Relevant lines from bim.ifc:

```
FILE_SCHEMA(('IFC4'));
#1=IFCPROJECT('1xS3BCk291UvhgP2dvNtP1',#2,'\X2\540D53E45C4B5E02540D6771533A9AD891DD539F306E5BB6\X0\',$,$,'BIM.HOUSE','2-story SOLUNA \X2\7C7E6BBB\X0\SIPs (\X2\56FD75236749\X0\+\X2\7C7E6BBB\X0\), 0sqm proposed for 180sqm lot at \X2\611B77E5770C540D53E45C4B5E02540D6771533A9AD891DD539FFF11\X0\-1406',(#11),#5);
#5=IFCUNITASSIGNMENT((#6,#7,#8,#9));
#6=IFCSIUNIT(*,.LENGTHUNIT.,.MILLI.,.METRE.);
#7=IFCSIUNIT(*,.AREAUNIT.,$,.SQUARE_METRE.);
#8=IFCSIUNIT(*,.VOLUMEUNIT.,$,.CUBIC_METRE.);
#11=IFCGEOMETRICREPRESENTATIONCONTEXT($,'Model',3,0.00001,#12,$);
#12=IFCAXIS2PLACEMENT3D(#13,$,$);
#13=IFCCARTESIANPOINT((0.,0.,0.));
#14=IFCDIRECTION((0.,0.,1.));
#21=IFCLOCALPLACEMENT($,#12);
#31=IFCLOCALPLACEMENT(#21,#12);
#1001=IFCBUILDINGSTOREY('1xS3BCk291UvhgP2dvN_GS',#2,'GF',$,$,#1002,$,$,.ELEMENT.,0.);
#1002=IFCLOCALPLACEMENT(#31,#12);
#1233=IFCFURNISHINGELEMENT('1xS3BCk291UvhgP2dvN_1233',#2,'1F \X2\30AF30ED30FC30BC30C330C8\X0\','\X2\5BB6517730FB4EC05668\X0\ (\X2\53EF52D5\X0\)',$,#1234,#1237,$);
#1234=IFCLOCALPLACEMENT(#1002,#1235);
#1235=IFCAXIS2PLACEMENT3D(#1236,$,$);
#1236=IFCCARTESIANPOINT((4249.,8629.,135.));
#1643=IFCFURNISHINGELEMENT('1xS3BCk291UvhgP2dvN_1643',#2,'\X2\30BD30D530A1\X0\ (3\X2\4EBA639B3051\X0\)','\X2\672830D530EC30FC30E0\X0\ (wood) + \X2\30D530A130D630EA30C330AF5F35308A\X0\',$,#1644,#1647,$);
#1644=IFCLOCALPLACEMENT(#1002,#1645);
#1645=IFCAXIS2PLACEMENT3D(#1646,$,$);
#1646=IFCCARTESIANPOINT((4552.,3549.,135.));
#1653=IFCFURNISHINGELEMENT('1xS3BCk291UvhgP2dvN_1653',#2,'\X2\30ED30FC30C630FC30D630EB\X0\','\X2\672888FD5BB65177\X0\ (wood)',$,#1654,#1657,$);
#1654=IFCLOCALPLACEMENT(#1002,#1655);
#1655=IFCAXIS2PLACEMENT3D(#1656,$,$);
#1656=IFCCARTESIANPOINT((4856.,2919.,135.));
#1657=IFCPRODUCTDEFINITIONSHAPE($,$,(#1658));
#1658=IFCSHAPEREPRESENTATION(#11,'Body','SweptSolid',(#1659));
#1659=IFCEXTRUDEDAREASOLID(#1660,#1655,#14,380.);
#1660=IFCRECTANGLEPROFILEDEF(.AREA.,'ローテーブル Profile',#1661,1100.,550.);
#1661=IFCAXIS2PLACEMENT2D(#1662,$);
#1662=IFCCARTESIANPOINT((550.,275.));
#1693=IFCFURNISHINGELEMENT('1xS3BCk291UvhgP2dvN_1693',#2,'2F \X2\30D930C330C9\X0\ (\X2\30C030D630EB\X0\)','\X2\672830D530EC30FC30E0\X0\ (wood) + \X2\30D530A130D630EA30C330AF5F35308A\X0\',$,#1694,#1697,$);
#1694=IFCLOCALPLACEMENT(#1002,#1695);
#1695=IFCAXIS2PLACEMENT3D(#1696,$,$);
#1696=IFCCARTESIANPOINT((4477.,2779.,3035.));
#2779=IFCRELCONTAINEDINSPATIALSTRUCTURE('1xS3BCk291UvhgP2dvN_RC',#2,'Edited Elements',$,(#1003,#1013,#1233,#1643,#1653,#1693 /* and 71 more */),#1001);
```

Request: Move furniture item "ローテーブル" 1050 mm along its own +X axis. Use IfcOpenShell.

```python
import ifcopenshell
import ifcopenshell.api.geometry
import ifcopenshell.util.placement
import ifcopenshell.util.unit

model = ifcopenshell.open("bim.ifc")
unit_scale = ifcopenshell.util.unit.calculate_unit_scale(model)

item = model.by_guid("1xS3BCk291UvhgP2dvN_1653")
matrix = ifcopenshell.util.placement.get_local_placement(item.ObjectPlacement)
matrix[:3, 3] += matrix[:3, 0] * 1.05 / unit_scale
ifcopenshell.api.geometry.edit_object_placement(model, product=item, matrix=matrix, is_si=False)

print(ifcopenshell.util.placement.get_local_placement(item.ObjectPlacement).round(3) + 0.0)

model.write("bim_updated.ifc")
```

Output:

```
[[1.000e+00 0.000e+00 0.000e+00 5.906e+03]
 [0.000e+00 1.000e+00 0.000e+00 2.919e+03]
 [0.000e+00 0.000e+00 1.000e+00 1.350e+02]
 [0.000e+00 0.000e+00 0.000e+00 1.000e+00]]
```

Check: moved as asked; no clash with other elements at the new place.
